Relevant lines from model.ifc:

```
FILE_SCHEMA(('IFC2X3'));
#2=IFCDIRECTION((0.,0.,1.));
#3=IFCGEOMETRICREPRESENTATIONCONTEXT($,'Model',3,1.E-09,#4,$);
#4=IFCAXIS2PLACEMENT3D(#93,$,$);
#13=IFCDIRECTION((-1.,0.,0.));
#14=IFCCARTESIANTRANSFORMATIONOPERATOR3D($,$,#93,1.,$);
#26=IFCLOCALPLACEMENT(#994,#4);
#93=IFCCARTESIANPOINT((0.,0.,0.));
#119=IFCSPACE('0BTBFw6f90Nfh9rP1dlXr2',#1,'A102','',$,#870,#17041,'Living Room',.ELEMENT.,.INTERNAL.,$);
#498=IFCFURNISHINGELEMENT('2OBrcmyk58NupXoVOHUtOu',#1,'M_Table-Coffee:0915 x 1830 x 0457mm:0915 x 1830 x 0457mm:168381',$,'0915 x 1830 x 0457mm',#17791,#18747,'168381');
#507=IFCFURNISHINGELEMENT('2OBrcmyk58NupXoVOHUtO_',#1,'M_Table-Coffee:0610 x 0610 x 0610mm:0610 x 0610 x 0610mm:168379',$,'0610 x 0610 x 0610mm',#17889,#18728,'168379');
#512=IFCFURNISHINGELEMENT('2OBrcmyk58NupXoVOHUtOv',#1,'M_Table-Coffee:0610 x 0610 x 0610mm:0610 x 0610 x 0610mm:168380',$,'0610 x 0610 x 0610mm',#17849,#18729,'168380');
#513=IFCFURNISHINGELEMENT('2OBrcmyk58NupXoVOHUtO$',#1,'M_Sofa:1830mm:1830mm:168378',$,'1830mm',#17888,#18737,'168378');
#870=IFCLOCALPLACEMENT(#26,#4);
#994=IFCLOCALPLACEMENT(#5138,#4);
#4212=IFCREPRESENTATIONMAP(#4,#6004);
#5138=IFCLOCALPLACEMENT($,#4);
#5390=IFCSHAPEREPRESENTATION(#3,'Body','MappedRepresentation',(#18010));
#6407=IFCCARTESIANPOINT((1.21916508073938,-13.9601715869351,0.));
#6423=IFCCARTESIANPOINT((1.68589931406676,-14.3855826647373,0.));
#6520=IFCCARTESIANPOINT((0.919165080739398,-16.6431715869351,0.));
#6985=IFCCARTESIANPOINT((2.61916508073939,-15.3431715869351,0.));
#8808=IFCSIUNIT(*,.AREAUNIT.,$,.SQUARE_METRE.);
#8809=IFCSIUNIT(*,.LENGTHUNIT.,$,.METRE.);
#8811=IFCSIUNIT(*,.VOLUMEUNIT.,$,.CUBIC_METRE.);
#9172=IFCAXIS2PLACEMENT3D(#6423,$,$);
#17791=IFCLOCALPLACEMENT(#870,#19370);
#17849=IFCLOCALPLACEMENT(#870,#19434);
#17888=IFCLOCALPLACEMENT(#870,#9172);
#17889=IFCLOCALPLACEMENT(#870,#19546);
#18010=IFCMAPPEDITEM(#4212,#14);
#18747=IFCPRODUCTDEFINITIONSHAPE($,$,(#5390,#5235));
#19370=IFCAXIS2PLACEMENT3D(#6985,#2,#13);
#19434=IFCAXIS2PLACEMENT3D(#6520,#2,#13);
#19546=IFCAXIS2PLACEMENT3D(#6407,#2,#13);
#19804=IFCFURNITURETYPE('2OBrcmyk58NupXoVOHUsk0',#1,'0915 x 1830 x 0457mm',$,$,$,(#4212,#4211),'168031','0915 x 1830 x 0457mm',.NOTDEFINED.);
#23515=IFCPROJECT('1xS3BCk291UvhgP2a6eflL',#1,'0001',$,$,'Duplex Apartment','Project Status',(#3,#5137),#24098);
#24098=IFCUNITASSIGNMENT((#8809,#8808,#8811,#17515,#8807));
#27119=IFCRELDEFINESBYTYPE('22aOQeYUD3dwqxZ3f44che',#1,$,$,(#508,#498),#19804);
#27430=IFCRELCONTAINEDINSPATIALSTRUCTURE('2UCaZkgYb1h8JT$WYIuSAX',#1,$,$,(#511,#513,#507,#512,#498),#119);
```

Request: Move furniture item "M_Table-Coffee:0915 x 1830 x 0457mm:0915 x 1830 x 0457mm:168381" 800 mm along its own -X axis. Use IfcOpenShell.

```python
import ifcopenshell
import ifcopenshell.api.geometry
import ifcopenshell.util.placement

model = ifcopenshell.open("model.ifc")

item = model.by_guid("2OBrcmyk58NupXoVOHUtOu")
matrix = ifcopenshell.util.placement.get_local_placement(item.ObjectPlacement)
matrix[:3, 3] -= matrix[:3, 0] * 0.8
ifcopenshell.api.geometry.edit_object_placement(model, product=item, matrix=matrix, is_si=False)

print(ifcopenshell.util.placement.get_local_placement(item.ObjectPlacement).round(3) + 0.0)

model.write("model_rev.ifc")
```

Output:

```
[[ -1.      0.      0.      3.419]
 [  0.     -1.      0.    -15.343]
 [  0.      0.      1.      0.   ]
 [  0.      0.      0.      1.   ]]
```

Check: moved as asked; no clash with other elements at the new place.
